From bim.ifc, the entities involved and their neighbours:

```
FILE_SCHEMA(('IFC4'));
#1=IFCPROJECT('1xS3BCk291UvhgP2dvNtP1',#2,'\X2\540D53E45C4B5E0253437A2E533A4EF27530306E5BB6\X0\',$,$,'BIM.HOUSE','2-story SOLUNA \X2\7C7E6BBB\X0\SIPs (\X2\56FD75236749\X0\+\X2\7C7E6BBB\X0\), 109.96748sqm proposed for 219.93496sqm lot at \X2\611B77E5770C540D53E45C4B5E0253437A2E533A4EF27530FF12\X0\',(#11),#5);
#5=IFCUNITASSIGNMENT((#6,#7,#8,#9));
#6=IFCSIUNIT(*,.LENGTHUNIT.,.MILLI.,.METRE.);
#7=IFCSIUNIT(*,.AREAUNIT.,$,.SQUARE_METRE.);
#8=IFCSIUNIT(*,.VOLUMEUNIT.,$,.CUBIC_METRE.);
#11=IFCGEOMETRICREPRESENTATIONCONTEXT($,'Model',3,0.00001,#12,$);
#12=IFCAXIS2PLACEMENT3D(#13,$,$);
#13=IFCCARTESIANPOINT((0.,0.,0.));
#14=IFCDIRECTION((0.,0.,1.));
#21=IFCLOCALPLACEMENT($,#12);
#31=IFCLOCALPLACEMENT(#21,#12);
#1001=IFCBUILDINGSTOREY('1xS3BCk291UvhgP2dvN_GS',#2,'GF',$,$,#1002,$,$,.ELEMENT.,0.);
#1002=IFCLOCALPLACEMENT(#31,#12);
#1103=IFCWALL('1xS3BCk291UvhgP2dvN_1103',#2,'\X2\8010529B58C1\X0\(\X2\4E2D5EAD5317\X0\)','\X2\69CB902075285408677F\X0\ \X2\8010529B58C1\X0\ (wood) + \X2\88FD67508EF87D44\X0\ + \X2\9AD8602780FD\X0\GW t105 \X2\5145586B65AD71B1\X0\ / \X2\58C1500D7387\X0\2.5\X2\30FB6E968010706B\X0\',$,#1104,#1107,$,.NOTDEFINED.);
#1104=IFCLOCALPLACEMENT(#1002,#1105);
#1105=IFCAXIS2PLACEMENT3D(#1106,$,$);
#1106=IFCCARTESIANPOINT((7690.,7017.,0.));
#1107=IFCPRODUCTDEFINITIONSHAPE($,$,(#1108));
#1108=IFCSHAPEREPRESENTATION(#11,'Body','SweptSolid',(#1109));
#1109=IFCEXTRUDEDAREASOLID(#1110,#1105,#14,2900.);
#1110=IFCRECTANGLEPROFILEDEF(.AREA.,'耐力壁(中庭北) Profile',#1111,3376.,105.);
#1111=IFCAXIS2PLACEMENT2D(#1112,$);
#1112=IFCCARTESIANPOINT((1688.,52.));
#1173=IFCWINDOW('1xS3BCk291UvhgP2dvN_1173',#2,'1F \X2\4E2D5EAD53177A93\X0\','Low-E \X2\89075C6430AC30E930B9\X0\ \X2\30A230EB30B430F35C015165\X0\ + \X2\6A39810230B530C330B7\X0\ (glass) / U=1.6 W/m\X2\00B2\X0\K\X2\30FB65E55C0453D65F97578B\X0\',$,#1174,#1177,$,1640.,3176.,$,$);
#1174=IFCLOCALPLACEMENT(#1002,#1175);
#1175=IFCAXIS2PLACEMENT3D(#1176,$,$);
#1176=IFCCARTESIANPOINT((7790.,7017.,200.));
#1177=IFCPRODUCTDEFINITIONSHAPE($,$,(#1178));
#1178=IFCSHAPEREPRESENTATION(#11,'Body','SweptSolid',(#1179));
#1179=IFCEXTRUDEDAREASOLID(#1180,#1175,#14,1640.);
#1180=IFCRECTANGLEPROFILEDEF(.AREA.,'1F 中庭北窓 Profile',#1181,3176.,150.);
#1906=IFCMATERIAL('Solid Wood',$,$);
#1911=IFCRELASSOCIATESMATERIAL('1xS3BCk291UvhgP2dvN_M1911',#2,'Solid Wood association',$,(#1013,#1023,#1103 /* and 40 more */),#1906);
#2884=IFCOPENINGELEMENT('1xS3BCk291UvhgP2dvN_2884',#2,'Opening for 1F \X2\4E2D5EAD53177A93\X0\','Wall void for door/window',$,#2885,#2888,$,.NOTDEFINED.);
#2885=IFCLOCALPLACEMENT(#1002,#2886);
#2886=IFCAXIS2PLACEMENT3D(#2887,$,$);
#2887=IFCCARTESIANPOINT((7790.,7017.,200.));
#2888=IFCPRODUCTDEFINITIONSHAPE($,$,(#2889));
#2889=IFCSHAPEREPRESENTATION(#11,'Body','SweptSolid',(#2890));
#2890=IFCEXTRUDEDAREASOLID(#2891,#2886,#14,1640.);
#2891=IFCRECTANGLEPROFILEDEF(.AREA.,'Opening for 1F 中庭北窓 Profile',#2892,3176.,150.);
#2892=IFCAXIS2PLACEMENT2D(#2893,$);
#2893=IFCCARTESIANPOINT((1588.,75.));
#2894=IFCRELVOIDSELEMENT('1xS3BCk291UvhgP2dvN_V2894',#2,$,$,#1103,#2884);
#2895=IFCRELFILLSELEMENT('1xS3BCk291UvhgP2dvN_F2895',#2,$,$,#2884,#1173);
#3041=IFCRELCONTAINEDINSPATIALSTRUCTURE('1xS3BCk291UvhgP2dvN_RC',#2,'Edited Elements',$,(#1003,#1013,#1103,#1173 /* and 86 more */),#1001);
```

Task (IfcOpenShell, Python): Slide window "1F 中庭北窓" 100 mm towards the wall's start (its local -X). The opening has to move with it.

```python
import ifcopenshell
import ifcopenshell.api.geometry
import ifcopenshell.util.placement
import ifcopenshell.util.unit

model = ifcopenshell.open("bim.ifc")
unit_scale = ifcopenshell.util.unit.calculate_unit_scale(model)

window = model.by_id(1173)
opening = window.FillsVoids[0].RelatingOpeningElement
wall = opening.VoidsElements[0].RelatingBuildingElement

wall_matrix = ifcopenshell.util.placement.get_local_placement(wall.ObjectPlacement)
shift = wall_matrix[:3, 0] * -0.1 / unit_scale
before = ifcopenshell.util.placement.get_local_placement(window.ObjectPlacement)[:3, 3].copy()

# The window is not placed relative to its opening, so move both.
for product in (opening, window):
    matrix = ifcopenshell.util.placement.get_local_placement(product.ObjectPlacement)
    matrix[:3, 3] += shift
    ifcopenshell.api.geometry.edit_object_placement(model, product=product, matrix=matrix, is_si=False)

after = ifcopenshell.util.placement.get_local_placement(window.ObjectPlacement)[:3, 3]
print("window moved by", (after - before).round(3) + 0.0)

model.write("bim_edited.ifc")
```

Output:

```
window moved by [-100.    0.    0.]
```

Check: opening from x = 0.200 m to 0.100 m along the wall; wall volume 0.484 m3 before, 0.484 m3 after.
